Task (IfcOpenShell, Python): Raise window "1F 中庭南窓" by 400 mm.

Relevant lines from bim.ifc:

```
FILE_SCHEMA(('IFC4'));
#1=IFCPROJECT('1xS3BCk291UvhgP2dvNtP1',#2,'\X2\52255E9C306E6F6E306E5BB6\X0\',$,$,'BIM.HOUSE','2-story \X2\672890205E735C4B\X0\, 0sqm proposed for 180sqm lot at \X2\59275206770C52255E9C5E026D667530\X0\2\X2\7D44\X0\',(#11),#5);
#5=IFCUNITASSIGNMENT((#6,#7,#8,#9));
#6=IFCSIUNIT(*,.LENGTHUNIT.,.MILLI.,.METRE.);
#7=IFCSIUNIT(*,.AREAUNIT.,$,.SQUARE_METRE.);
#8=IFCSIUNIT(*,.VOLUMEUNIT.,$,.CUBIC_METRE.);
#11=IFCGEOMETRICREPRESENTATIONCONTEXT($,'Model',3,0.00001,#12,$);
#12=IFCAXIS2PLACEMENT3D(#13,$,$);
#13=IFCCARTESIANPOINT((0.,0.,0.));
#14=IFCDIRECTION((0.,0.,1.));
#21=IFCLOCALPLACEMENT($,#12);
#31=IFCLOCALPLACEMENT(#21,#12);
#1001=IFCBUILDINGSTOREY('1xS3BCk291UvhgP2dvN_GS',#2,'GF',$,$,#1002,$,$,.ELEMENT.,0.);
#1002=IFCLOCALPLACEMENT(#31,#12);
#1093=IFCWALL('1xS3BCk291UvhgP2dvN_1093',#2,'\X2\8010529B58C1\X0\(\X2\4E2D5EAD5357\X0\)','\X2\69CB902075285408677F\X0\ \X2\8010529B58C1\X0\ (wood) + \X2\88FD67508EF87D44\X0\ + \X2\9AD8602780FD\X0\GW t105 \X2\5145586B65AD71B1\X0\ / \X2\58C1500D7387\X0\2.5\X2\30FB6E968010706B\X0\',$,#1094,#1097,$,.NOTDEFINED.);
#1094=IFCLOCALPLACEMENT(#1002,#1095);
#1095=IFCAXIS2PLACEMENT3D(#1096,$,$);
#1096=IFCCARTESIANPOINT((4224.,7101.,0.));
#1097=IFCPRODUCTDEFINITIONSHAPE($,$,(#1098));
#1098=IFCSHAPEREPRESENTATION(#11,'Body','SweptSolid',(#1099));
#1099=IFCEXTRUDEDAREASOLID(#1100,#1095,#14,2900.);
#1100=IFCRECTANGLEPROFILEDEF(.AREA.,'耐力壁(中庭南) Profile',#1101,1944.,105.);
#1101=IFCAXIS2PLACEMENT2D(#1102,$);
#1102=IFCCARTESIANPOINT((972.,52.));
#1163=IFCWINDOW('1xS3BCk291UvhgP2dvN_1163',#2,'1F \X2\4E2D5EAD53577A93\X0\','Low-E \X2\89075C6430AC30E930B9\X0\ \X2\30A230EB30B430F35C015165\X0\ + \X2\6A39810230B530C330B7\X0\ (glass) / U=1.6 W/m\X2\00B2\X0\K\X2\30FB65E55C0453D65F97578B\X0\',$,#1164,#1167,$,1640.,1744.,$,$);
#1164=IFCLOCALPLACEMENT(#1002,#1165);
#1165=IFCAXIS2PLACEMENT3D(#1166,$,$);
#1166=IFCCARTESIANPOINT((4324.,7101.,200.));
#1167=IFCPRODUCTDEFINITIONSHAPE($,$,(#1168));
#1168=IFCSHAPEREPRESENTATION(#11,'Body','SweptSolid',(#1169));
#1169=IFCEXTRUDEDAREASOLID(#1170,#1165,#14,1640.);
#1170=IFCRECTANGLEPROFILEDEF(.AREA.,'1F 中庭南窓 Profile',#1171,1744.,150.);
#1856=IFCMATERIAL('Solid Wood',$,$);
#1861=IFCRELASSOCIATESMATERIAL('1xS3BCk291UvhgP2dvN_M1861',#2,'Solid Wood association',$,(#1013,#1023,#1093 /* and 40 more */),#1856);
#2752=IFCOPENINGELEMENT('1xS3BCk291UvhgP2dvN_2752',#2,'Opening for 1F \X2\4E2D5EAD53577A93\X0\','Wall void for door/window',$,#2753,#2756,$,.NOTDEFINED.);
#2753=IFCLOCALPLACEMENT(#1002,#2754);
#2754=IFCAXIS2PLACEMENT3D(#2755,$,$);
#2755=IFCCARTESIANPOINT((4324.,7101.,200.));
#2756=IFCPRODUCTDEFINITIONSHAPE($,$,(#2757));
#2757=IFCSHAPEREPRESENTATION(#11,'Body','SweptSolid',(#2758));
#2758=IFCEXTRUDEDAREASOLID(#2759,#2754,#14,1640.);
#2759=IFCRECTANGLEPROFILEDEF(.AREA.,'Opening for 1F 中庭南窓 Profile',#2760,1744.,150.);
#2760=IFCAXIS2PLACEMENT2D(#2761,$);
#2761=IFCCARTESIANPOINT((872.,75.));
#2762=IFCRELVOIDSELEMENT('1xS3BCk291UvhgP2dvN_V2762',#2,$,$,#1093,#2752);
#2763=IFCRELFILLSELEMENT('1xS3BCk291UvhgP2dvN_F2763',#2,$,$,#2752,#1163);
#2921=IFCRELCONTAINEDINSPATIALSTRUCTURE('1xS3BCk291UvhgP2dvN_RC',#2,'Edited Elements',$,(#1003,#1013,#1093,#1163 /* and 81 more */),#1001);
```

```python
import numpy as np
import ifcopenshell
import ifcopenshell.api.geometry
import ifcopenshell.util.placement
import ifcopenshell.util.unit

model = ifcopenshell.open("bim.ifc")
unit_scale = ifcopenshell.util.unit.calculate_unit_scale(model)

window = model.by_guid("1xS3BCk291UvhgP2dvN_1163")
opening = window.FillsVoids[0].RelatingOpeningElement
dz = 0.4 / unit_scale

shift = np.array([0.0, 0.0, dz])
# The window is not placed relative to its opening, so move both.
for product in (opening, window):
    matrix = ifcopenshell.util.placement.get_local_placement(product.ObjectPlacement)
    matrix[:3, 3] += shift
    ifcopenshell.api.geometry.edit_object_placement(model, product=product, matrix=matrix, is_si=False)

print(f"moved by {dz * unit_scale:+.3f} m")

model.write("bim_rev.ifc")
```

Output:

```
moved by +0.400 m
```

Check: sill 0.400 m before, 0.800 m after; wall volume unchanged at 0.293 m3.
